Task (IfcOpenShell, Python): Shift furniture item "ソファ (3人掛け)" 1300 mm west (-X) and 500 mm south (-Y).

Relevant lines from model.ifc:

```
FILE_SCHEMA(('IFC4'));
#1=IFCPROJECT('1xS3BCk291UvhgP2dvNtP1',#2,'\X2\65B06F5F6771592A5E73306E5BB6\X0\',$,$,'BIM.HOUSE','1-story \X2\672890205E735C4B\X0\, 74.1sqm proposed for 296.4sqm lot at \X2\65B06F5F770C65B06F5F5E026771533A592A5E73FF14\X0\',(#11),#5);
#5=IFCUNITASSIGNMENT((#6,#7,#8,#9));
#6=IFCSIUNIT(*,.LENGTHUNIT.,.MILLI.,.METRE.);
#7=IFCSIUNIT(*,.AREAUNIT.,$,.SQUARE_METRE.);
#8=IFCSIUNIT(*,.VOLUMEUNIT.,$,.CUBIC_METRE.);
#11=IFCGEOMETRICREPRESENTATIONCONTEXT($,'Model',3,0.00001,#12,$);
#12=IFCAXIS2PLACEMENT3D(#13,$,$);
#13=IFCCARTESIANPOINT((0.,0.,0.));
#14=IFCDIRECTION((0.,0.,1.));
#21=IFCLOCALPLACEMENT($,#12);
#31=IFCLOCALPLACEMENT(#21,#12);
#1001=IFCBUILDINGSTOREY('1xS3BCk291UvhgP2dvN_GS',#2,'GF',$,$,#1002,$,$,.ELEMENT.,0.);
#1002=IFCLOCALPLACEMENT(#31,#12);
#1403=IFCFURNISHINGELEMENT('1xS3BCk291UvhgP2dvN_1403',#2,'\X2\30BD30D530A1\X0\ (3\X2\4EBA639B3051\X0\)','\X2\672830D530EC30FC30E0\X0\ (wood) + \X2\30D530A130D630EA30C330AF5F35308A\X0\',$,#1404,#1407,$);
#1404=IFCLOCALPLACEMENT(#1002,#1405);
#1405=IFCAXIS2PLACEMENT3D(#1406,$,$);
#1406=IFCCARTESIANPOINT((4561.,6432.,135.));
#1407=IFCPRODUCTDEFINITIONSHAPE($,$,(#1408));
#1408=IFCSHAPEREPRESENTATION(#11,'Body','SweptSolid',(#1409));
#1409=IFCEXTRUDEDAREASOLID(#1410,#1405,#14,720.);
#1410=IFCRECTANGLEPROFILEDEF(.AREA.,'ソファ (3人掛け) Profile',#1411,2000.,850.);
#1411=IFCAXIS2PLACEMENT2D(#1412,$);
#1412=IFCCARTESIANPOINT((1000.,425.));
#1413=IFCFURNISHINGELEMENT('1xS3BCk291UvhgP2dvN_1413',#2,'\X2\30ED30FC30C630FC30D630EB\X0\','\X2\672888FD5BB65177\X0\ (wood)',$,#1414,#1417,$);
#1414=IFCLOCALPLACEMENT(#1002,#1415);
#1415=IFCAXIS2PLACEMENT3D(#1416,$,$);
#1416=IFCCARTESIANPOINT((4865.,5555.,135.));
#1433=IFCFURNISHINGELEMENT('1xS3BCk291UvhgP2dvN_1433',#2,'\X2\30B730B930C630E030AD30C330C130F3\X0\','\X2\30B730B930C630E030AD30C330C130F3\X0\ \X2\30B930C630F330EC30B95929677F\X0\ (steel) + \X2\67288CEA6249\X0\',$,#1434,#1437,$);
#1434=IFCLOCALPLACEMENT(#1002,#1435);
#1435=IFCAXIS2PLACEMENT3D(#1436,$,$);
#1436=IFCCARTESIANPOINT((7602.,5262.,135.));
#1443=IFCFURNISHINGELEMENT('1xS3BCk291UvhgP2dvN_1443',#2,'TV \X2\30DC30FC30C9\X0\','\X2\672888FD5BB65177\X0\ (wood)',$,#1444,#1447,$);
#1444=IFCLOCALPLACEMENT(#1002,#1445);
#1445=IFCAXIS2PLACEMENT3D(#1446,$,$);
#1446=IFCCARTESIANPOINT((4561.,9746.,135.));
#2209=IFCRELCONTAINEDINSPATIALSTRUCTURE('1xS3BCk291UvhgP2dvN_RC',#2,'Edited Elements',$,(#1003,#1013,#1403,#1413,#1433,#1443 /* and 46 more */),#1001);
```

```python
import ifcopenshell
import ifcopenshell.api.geometry
import ifcopenshell.util.placement
import ifcopenshell.util.unit

model = ifcopenshell.open("model.ifc")
unit_scale = ifcopenshell.util.unit.calculate_unit_scale(model)

item = model.by_guid("1xS3BCk291UvhgP2dvN_1403")
matrix = ifcopenshell.util.placement.get_local_placement(item.ObjectPlacement)
matrix[0, 3] -= 1.3 / unit_scale
matrix[1, 3] -= 0.5 / unit_scale
ifcopenshell.api.geometry.edit_object_placement(model, product=item, matrix=matrix, is_si=False)

print(ifcopenshell.util.placement.get_local_placement(item.ObjectPlacement).round(3) + 0.0)

model.write("model_edited.ifc")
```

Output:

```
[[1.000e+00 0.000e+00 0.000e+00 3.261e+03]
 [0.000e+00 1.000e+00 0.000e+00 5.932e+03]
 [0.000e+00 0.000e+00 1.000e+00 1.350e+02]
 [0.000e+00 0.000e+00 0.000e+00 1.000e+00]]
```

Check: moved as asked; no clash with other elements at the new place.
